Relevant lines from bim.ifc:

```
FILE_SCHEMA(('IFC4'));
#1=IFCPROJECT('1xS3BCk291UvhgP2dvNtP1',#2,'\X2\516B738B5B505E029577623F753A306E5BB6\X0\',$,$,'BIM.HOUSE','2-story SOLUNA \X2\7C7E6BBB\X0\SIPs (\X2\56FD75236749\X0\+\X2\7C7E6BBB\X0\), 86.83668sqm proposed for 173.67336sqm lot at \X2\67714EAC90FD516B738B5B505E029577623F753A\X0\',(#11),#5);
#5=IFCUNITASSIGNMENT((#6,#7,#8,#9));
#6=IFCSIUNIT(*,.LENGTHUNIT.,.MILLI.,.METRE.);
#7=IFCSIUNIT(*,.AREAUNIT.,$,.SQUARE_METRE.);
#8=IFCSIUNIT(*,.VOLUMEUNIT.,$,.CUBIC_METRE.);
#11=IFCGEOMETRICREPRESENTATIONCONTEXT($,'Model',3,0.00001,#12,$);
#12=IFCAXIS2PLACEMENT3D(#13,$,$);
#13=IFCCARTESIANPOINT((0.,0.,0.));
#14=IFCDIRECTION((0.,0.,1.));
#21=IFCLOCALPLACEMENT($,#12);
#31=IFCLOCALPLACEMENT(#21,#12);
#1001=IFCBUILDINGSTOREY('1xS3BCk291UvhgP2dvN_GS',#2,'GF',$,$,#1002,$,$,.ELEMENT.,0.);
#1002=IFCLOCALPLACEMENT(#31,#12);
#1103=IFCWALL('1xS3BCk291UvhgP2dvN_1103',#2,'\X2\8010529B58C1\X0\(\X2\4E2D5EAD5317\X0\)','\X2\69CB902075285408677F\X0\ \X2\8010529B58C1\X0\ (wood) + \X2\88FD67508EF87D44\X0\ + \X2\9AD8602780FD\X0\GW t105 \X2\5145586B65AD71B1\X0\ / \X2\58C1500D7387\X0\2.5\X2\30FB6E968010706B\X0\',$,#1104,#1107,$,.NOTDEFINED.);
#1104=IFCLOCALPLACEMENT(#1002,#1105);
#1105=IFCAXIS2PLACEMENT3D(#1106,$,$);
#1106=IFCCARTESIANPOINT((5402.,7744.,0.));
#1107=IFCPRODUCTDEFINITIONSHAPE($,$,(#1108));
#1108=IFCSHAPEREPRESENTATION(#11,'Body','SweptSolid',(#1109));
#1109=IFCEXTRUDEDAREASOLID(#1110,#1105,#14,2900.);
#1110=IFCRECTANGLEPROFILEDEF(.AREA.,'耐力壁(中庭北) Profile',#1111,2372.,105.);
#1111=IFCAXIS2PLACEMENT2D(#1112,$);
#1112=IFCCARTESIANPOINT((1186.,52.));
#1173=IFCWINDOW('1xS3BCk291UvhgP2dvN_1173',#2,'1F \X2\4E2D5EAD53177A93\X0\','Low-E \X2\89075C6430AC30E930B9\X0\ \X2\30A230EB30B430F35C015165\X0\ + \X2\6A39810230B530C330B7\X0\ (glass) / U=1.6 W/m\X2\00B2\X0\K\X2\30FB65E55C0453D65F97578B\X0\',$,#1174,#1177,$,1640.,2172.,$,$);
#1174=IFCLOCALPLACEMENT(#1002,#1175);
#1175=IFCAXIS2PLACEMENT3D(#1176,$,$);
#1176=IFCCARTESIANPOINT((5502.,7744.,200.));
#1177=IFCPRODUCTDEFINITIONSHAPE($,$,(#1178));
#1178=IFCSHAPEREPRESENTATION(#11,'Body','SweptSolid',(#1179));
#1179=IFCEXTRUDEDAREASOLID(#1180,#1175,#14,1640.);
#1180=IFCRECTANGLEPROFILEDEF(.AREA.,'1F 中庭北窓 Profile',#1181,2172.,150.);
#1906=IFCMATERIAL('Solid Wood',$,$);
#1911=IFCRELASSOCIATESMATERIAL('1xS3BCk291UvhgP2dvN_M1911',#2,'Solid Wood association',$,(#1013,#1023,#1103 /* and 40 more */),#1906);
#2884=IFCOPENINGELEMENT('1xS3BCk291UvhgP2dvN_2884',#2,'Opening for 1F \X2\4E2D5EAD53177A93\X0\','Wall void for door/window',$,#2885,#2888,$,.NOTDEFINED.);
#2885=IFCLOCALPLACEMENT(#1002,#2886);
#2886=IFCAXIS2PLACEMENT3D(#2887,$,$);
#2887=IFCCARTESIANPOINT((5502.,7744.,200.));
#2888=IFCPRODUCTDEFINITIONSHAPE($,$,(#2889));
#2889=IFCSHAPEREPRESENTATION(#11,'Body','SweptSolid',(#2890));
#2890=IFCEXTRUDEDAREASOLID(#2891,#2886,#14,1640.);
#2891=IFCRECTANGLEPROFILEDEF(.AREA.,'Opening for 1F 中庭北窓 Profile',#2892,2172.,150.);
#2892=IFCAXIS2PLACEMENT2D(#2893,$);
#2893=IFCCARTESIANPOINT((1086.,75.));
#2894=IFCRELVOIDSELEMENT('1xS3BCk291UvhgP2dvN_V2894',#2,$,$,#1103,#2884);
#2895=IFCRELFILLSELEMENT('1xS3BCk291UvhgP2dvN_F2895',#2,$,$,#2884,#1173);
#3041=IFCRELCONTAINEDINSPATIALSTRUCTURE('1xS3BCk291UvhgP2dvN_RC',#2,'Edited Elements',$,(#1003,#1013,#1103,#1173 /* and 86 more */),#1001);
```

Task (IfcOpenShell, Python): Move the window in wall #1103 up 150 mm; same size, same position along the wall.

```python
import numpy as np
import ifcopenshell
import ifcopenshell.api.geometry
import ifcopenshell.util.placement
import ifcopenshell.util.unit

model = ifcopenshell.open("bim.ifc")
unit_scale = ifcopenshell.util.unit.calculate_unit_scale(model)

window = model.by_guid("1xS3BCk291UvhgP2dvN_1173")
opening = window.FillsVoids[0].RelatingOpeningElement
dz = 0.15 / unit_scale

shift = np.array([0.0, 0.0, dz])
# The window is not placed relative to its opening, so move both.
for product in (opening, window):
    matrix = ifcopenshell.util.placement.get_local_placement(product.ObjectPlacement)
    matrix[:3, 3] += shift
    ifcopenshell.api.geometry.edit_object_placement(model, product=product, matrix=matrix, is_si=False)

print(f"moved by {dz * unit_scale:+.3f} m")

model.write("bim_edited.ifc")
```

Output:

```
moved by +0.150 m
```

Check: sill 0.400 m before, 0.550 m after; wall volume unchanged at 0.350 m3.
